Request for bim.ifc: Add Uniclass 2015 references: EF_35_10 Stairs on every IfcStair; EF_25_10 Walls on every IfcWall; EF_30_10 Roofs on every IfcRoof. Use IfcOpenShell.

First a look at what the model holds.

```python
import ifcopenshell

model = ifcopenshell.open("bim.ifc")
print(model.schema)
print("classifications:", [c.Name for c in model.by_type("IfcClassification")])
for ifc_class in ("IfcDoor", "IfcRoof", "IfcStair", "IfcWall", "IfcWindow"):
    print(ifc_class, len(model.by_type(ifc_class)))
```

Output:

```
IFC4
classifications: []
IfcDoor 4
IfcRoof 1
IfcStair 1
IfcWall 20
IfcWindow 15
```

```python
import ifcopenshell
import ifcopenshell.api.classification

model = ifcopenshell.open("bim.ifc")

system = ifcopenshell.api.classification.add_classification(model, classification="Uniclass 2015")

codes = {
    "IfcStair": ("EF_35_10", "Stairs"),
    "IfcWall": ("EF_25_10", "Walls"),
    "IfcRoof": ("EF_30_10", "Roofs"),
}
for ifc_class, (code, name) in codes.items():
    products = model.by_type(ifc_class)
    ifcopenshell.api.classification.add_reference(
        model, products=products, classification=system, identification=code, name=name
    )
    print(code, len(products))

model.write("bim_updated.ifc")
```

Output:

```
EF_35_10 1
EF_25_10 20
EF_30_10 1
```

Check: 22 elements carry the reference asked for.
